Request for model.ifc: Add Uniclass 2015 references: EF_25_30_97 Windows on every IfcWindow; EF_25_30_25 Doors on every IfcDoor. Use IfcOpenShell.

First a look at what the model holds.

```python
import ifcopenshell

model = ifcopenshell.open("model.ifc")
print(model.schema)
print("classifications:", [c.Name for c in model.by_type("IfcClassification")])
for ifc_class in ("IfcDoor", "IfcRoof", "IfcStair", "IfcWall", "IfcWindow"):
    print(ifc_class, len(model.by_type(ifc_class)))
```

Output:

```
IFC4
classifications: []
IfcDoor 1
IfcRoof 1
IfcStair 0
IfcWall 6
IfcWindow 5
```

```python
import ifcopenshell
import ifcopenshell.api.classification

model = ifcopenshell.open("model.ifc")

system = ifcopenshell.api.classification.add_classification(model, classification="Uniclass 2015")

codes = {
    "IfcWindow": ("EF_25_30_97", "Windows"),
    "IfcDoor": ("EF_25_30_25", "Doors"),
}
for ifc_class, (code, name) in codes.items():
    products = model.by_type(ifc_class)
    ifcopenshell.api.classification.add_reference(
        model, products=products, classification=system, identification=code, name=name
    )
    print(code, len(products))

model.write("model-out.ifc")
```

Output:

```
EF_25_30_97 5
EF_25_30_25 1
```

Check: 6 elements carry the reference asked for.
